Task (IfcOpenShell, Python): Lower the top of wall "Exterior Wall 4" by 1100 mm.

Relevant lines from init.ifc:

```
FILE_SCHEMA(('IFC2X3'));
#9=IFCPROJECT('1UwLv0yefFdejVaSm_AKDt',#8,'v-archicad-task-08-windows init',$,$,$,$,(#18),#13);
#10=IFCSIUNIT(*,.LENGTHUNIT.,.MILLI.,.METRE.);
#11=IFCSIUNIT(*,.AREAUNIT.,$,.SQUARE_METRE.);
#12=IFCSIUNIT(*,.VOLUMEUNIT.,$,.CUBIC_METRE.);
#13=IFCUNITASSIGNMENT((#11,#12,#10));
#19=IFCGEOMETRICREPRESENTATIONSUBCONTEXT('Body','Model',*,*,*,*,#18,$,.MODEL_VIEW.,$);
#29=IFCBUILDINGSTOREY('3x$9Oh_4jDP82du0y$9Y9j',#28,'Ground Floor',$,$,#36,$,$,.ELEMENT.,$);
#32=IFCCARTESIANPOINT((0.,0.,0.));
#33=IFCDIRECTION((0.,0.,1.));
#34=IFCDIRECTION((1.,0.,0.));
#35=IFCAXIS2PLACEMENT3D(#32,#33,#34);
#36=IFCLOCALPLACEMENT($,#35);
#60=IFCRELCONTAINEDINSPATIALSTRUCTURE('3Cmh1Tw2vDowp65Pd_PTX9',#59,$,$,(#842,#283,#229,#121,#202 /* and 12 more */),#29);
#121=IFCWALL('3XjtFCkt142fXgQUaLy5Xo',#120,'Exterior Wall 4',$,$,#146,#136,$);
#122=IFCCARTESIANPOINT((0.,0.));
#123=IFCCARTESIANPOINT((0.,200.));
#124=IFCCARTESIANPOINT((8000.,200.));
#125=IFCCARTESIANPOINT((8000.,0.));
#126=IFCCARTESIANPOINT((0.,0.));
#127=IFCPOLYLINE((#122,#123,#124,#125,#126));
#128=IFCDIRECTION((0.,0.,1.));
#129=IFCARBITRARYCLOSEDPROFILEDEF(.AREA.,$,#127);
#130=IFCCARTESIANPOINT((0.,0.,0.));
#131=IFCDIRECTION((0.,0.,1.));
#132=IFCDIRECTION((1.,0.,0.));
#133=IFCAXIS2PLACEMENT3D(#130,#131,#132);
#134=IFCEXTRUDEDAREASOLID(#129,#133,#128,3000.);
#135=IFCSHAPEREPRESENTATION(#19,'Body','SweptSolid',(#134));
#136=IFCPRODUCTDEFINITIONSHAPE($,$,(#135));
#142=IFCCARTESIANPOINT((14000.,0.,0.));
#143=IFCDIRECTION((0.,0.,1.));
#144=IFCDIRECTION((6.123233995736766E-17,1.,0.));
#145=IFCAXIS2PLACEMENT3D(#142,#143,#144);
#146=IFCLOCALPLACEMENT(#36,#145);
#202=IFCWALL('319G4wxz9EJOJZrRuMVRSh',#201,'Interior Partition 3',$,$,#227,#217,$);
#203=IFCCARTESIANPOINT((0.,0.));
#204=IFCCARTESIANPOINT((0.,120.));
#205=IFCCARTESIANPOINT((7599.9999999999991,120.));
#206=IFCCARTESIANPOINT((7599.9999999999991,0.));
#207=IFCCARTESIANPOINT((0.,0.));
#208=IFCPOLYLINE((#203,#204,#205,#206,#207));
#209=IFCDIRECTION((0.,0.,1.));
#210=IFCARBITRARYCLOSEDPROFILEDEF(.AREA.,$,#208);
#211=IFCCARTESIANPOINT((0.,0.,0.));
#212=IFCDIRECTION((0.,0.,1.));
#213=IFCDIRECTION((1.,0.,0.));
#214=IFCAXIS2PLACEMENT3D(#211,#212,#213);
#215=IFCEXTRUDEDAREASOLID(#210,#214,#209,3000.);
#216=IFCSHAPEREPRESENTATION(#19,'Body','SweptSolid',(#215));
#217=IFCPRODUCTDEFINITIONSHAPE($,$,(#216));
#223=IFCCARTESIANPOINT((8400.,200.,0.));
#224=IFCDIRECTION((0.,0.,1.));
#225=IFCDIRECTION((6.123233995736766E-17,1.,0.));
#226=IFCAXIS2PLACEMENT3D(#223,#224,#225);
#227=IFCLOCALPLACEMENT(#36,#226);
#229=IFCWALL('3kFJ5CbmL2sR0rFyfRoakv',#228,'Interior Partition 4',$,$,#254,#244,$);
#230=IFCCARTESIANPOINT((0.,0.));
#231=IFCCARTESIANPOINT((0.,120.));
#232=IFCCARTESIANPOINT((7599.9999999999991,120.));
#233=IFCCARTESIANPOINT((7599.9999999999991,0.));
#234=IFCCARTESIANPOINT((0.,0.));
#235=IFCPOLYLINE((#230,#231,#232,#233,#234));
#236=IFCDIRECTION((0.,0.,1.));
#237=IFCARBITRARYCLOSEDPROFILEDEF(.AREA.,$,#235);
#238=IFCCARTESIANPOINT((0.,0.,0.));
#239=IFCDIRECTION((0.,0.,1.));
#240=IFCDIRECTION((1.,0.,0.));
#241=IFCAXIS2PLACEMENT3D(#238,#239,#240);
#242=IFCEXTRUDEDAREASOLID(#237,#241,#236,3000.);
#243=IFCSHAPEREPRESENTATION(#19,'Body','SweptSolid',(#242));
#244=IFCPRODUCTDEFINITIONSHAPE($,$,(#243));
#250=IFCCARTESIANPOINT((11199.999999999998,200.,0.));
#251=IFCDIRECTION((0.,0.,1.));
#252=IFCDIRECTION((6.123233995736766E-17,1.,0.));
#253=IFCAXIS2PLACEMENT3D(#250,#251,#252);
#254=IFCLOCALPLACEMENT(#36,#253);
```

```python
import ifcopenshell
import ifcopenshell.geom
import ifcopenshell.util.representation
import ifcopenshell.util.shape

model = ifcopenshell.open("init.ifc")
settings = ifcopenshell.geom.settings()


def volume(element):
    """Net volume in cubic metres, openings subtracted."""
    shape = ifcopenshell.geom.create_shape(settings, element)
    return ifcopenshell.util.shape.get_volume(shape.geometry)


wall = model.by_guid("3XjtFCkt142fXgQUaLy5Xo")
before = volume(wall)

body = ifcopenshell.util.representation.get_representation(wall, "Model", "Body")
solid = body.Items[0]
old_height = solid.Depth
solid.Depth -= 1100.0
after = volume(wall)

print(f"height {old_height:g} -> {solid.Depth:g}, volume {before:.3f} -> {after:.3f} m3")

model.write("init_v2.ifc")
```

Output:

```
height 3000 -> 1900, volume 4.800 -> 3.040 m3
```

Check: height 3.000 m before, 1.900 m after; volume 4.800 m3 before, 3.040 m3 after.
